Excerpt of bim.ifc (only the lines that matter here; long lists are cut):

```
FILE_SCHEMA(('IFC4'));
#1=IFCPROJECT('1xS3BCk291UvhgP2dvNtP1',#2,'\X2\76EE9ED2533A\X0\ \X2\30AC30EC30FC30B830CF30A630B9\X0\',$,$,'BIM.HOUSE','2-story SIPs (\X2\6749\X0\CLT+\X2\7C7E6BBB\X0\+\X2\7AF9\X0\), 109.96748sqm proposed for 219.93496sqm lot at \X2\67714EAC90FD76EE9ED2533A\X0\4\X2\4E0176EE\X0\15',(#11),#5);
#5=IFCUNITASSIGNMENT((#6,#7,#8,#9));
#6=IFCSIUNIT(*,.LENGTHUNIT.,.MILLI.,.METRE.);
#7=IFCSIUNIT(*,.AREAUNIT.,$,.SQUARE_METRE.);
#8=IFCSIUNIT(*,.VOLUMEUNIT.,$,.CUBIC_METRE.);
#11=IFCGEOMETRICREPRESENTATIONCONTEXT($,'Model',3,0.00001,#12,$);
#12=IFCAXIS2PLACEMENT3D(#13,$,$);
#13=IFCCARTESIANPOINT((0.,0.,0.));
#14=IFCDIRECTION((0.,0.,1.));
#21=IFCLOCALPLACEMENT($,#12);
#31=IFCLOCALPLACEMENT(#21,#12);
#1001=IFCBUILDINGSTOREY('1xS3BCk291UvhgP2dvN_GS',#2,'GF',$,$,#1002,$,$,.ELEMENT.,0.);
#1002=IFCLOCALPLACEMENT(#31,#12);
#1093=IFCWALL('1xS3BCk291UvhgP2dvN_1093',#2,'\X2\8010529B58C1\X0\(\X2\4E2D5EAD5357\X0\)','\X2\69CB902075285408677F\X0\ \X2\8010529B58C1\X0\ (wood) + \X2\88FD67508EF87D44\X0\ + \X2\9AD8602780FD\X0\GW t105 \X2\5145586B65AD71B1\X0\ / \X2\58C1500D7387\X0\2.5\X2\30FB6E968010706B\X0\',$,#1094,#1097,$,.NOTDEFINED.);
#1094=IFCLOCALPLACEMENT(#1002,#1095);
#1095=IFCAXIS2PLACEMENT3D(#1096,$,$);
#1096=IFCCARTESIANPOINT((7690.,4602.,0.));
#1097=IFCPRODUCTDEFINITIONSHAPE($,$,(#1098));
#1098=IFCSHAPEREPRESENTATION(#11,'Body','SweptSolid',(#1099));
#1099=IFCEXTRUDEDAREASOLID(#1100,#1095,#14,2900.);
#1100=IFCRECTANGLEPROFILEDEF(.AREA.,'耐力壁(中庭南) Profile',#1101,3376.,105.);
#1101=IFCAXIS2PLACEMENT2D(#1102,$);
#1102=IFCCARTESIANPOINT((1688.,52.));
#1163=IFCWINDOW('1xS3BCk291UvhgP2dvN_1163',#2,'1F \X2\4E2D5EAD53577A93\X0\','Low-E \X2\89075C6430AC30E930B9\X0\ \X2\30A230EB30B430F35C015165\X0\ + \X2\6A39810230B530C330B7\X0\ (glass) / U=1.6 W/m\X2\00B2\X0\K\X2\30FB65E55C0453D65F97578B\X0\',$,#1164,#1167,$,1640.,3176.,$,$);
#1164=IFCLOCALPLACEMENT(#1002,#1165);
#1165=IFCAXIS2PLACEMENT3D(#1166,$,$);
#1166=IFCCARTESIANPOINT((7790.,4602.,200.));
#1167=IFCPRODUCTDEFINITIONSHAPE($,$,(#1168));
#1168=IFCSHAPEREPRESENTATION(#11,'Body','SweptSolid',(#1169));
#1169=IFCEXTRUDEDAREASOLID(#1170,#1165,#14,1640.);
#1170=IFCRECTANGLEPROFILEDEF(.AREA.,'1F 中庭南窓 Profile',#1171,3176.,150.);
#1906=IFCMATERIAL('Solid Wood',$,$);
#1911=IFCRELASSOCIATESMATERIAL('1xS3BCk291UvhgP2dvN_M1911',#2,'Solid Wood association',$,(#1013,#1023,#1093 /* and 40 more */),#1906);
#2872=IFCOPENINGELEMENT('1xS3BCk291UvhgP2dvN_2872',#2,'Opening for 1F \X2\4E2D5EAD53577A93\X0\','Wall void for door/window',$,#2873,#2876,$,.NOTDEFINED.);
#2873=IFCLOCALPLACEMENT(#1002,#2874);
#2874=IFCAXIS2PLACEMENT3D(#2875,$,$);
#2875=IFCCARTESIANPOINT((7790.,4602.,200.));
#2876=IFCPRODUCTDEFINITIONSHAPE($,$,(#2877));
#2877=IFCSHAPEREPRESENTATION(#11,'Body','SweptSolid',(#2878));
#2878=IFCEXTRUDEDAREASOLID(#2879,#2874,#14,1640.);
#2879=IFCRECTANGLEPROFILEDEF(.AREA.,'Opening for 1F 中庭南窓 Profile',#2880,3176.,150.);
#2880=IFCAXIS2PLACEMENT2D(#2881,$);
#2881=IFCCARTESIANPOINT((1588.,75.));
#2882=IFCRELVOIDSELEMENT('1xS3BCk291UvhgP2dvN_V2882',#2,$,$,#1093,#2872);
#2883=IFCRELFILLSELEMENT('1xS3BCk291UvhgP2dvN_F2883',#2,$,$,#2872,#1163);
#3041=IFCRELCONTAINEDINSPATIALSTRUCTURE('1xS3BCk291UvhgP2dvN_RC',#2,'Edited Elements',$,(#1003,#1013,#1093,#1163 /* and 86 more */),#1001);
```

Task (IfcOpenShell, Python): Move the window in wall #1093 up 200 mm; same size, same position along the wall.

```python
import numpy as np
import ifcopenshell
import ifcopenshell.api.geometry
import ifcopenshell.util.placement
import ifcopenshell.util.unit

model = ifcopenshell.open("bim.ifc")
unit_scale = ifcopenshell.util.unit.calculate_unit_scale(model)

window = model.by_id(1163)
opening = window.FillsVoids[0].RelatingOpeningElement
dz = 200.0

shift = np.array([0.0, 0.0, dz])
# The window is not placed relative to its opening, so move both.
for product in (opening, window):
    matrix = ifcopenshell.util.placement.get_local_placement(product.ObjectPlacement)
    matrix[:3, 3] += shift
    ifcopenshell.api.geometry.edit_object_placement(model, product=product, matrix=matrix, is_si=False)

print(f"moved by {dz * unit_scale:+.3f} m")

model.write("bim_updated.ifc")
```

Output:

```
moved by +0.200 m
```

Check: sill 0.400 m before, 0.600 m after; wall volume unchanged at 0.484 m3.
